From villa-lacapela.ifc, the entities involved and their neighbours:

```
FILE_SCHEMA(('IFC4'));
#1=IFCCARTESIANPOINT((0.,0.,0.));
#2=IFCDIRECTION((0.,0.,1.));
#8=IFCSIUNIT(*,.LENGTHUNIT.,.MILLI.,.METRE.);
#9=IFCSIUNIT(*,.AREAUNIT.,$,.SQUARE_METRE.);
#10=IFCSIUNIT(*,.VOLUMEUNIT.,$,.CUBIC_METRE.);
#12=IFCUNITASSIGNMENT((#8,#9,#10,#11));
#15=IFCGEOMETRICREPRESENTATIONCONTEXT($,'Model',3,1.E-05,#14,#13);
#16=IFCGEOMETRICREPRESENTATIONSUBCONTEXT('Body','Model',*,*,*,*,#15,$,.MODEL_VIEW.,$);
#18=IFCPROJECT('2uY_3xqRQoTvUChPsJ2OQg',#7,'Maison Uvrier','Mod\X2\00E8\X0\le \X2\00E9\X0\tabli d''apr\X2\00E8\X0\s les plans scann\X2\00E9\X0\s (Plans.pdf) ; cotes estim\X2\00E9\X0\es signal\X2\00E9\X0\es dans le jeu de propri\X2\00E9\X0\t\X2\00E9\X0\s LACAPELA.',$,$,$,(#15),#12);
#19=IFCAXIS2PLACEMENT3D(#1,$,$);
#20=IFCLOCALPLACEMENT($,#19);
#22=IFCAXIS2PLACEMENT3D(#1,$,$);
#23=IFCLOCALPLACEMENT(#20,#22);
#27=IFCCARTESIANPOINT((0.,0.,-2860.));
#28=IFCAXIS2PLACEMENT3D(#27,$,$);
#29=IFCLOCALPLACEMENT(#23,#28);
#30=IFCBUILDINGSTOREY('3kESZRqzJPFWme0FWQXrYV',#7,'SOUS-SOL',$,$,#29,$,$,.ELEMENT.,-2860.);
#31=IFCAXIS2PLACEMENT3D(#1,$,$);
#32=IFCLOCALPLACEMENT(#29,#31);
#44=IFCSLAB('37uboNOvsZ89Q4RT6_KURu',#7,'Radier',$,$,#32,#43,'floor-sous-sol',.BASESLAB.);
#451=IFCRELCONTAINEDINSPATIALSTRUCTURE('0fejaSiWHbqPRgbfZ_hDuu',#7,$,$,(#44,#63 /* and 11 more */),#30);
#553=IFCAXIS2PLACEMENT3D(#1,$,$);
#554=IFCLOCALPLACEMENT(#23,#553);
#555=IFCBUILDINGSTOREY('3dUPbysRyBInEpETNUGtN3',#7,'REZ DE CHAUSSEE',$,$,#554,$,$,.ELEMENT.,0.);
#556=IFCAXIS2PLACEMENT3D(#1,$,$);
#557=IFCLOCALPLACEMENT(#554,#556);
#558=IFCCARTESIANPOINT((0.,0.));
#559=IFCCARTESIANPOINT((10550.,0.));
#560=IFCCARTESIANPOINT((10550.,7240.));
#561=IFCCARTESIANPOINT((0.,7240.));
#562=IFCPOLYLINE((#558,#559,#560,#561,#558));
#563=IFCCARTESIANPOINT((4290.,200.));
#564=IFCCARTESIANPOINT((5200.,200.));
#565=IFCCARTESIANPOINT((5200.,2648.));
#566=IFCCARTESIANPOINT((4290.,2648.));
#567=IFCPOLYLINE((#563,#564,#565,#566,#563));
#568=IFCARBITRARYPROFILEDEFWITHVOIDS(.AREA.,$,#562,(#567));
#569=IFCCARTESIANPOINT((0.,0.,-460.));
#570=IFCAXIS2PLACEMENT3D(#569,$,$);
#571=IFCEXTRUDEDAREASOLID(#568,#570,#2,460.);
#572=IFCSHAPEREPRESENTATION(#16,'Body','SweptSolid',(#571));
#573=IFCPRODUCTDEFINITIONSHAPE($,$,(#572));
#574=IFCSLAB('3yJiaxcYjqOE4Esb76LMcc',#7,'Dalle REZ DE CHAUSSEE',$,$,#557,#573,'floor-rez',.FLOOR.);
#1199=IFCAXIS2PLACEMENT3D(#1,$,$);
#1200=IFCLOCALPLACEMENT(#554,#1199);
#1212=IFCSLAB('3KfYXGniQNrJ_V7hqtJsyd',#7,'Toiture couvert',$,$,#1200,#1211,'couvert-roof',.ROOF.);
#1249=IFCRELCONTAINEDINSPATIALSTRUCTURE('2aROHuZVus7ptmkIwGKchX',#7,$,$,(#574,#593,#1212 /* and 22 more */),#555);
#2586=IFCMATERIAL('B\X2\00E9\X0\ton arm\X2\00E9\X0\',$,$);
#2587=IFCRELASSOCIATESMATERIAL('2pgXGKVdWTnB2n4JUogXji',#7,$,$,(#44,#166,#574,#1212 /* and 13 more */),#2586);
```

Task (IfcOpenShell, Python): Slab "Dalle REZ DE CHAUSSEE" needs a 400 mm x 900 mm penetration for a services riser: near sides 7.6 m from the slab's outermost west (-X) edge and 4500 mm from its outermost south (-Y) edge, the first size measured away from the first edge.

```python
import numpy as np
import ifcopenshell
import ifcopenshell.api.feature
import ifcopenshell.api.geometry
import ifcopenshell.api.root
import ifcopenshell.geom
import ifcopenshell.util.placement
import ifcopenshell.util.representation
import ifcopenshell.util.shape
import ifcopenshell.util.unit

model = ifcopenshell.open("villa-lacapela.ifc")
unit_scale = ifcopenshell.util.unit.calculate_unit_scale(model)
settings = ifcopenshell.geom.settings()


def volume(element):
    """Net volume in cubic metres, openings subtracted."""
    shape = ifcopenshell.geom.create_shape(settings, element)
    return ifcopenshell.util.shape.get_volume(shape.geometry)


slab = model.by_id(574)
before = volume(slab)

# Extent in the slab's own axes, in metres. The edges named are its -X and -Y sides.
slab_shape = ifcopenshell.geom.create_shape(settings, slab)
vertices = ifcopenshell.util.shape.get_vertices(slab_shape.geometry)
x_min, y_min, bottom = vertices.min(axis=0)
top = vertices[:, 2].max()

opening = ifcopenshell.api.root.create_entity(model, ifc_class="IfcOpeningElement", name="Services riser opening", predefined_type="OPENING")
context = ifcopenshell.util.representation.get_context(model, "Model", "Body", "MODEL_VIEW")
width, depth = 0.4, 0.9
outline = [(0.0, 0.0), (width, 0.0), (width, depth), (0.0, depth), (0.0, 0.0)]
# Overshoot both faces by 50 mm so the cut is clean.
shape = ifcopenshell.api.geometry.add_slab_representation(
    model, context=context, depth=top - bottom + 0.1, polyline=outline
)
ifcopenshell.api.geometry.assign_representation(model, product=opening, representation=shape)

matrix = ifcopenshell.util.placement.get_local_placement(slab.ObjectPlacement)
matrix[:, 3] = matrix @ np.append(np.array([x_min + 7.6, y_min + 4.5, bottom - 0.05]) / unit_scale, 1.0)
ifcopenshell.api.geometry.edit_object_placement(model, product=opening, matrix=matrix, is_si=False)
ifcopenshell.api.feature.add_feature(model, feature=opening, element=slab)

after = volume(slab)

print(f"slab volume {before:.3f} -> {after:.3f} m3")

model.write("villa-lacapela_v2.ifc")
```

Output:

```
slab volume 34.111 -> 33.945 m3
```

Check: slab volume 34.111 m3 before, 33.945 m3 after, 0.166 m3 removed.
